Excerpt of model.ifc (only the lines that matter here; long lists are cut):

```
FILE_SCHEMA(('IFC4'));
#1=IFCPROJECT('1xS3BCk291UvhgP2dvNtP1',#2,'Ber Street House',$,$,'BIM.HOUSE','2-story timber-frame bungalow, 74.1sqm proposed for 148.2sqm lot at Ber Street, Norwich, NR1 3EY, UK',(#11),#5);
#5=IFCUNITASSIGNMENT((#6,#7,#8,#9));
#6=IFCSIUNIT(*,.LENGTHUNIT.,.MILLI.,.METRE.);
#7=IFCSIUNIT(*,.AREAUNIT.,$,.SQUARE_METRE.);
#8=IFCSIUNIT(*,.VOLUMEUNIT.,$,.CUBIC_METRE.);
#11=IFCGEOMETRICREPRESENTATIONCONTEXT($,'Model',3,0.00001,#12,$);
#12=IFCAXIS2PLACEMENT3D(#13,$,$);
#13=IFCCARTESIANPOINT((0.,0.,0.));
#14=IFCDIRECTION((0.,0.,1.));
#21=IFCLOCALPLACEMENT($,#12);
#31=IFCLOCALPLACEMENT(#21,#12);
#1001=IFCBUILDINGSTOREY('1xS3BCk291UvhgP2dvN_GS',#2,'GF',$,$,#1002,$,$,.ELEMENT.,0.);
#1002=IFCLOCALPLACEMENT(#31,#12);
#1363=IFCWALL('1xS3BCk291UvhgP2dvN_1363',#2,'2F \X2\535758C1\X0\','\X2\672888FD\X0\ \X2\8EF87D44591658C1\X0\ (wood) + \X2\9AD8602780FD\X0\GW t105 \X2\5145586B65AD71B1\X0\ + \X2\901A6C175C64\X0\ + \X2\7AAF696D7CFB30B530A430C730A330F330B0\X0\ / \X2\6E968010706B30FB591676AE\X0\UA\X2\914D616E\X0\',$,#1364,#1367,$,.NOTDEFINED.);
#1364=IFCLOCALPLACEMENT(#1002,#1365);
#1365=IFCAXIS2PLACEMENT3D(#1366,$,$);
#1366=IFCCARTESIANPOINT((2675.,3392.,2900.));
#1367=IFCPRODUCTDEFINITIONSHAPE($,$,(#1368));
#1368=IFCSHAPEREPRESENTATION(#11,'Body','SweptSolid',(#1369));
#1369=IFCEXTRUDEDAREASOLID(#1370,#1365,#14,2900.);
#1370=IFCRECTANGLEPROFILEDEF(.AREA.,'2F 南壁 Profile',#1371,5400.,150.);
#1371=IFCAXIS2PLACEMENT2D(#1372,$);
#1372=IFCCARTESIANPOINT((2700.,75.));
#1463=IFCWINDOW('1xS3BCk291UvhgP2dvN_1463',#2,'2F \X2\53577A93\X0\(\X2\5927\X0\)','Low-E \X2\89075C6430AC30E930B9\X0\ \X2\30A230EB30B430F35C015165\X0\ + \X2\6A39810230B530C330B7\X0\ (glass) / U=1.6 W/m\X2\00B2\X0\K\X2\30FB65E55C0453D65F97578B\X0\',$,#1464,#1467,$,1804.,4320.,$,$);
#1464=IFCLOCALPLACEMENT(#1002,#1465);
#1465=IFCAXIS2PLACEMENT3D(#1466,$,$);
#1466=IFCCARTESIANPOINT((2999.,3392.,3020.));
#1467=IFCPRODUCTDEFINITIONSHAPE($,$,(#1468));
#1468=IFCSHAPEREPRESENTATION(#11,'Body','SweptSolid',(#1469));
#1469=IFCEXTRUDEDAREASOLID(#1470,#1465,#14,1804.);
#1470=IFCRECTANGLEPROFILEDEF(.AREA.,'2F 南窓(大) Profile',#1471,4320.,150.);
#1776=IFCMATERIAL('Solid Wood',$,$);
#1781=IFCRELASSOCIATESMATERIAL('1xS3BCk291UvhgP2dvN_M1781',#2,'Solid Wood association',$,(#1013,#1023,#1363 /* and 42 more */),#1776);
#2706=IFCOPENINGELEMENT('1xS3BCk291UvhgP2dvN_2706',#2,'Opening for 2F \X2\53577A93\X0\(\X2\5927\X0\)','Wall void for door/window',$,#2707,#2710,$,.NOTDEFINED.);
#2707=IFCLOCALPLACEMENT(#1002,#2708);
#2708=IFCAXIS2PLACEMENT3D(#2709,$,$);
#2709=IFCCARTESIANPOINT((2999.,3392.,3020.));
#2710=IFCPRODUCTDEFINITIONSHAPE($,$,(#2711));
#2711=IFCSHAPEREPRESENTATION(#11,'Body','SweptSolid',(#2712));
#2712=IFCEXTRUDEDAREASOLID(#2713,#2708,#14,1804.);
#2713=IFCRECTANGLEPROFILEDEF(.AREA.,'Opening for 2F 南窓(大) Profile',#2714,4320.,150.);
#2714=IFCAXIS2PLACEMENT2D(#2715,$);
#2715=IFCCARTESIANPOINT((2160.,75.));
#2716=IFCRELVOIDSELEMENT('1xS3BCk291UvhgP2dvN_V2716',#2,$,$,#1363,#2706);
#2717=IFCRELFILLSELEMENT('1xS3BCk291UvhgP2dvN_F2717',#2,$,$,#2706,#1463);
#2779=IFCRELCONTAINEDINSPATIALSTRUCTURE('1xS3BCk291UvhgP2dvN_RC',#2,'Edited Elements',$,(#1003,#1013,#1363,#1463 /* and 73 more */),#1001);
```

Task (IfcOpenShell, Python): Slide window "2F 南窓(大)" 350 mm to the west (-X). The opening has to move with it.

```python
import ifcopenshell
import ifcopenshell.api.geometry
import ifcopenshell.util.placement

model = ifcopenshell.open("model.ifc")

window = model.by_id(1463)
opening = window.FillsVoids[0].RelatingOpeningElement
wall = opening.VoidsElements[0].RelatingBuildingElement

wall_matrix = ifcopenshell.util.placement.get_local_placement(wall.ObjectPlacement)
shift = wall_matrix[:3, 0] * -350.0
before = ifcopenshell.util.placement.get_local_placement(window.ObjectPlacement)[:3, 3].copy()

# The window is not placed relative to its opening, so move both.
for product in (opening, window):
    matrix = ifcopenshell.util.placement.get_local_placement(product.ObjectPlacement)
    matrix[:3, 3] += shift
    ifcopenshell.api.geometry.edit_object_placement(model, product=product, matrix=matrix, is_si=False)

after = ifcopenshell.util.placement.get_local_placement(window.ObjectPlacement)[:3, 3]
print("window moved by", (after - before).round(3) + 0.0)

model.write("model_v2.ifc")
```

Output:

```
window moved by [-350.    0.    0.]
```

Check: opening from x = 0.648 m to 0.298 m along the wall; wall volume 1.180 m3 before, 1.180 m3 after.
